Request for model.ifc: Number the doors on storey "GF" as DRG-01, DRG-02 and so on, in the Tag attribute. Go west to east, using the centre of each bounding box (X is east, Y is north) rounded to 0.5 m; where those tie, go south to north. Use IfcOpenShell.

First a look at what the model holds.

```python
import ifcopenshell
import ifcopenshell.util.element
import ifcopenshell.util.placement

model = ifcopenshell.open("model.ifc")
print(model.schema)
storey = next(s for s in model.by_type("IfcBuildingStorey") if s.Name == "GF")
doors = [e for e in ifcopenshell.util.element.get_decomposition(storey) if e.is_a("IfcDoor")]
for e in sorted(doors, key=lambda e: e.id()):
    origin = ifcopenshell.util.placement.get_local_placement(e.ObjectPlacement)[:3, 3]
    print(e.id(), e.Tag, e.Name, origin.round(2) + 0.0, sep=" | ")
```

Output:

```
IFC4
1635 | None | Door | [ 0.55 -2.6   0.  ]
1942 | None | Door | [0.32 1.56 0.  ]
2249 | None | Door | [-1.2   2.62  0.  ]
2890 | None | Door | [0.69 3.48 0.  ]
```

```python
import ifcopenshell
import ifcopenshell.geom
import ifcopenshell.util.element
import ifcopenshell.util.shape

model = ifcopenshell.open("model.ifc")
settings = ifcopenshell.geom.settings()
settings.set("use-world-coords", True)


def centre(element):
    shape = ifcopenshell.geom.create_shape(settings, element)
    return ifcopenshell.util.shape.get_bbox_centroid(shape.geometry)


storey = next(s for s in model.by_type("IfcBuildingStorey") if s.Name == "GF")
doors = [e for e in ifcopenshell.util.element.get_decomposition(storey) if e.is_a("IfcDoor")]

# Insertion points can sit at a corner or the storey origin, so sort by the geometry (in metres).
centres = {e: centre(e) for e in doors}
doors.sort(key=lambda e: (round(centres[e][0] / 0.5), centres[e][1]))

for i, e in enumerate(doors, start=1):
    number = f"DRG-{i:02d}"
    e.Tag = number
    print(e.id(), number)

model.write("model_edited.ifc")
```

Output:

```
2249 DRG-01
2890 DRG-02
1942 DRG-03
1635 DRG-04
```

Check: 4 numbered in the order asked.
